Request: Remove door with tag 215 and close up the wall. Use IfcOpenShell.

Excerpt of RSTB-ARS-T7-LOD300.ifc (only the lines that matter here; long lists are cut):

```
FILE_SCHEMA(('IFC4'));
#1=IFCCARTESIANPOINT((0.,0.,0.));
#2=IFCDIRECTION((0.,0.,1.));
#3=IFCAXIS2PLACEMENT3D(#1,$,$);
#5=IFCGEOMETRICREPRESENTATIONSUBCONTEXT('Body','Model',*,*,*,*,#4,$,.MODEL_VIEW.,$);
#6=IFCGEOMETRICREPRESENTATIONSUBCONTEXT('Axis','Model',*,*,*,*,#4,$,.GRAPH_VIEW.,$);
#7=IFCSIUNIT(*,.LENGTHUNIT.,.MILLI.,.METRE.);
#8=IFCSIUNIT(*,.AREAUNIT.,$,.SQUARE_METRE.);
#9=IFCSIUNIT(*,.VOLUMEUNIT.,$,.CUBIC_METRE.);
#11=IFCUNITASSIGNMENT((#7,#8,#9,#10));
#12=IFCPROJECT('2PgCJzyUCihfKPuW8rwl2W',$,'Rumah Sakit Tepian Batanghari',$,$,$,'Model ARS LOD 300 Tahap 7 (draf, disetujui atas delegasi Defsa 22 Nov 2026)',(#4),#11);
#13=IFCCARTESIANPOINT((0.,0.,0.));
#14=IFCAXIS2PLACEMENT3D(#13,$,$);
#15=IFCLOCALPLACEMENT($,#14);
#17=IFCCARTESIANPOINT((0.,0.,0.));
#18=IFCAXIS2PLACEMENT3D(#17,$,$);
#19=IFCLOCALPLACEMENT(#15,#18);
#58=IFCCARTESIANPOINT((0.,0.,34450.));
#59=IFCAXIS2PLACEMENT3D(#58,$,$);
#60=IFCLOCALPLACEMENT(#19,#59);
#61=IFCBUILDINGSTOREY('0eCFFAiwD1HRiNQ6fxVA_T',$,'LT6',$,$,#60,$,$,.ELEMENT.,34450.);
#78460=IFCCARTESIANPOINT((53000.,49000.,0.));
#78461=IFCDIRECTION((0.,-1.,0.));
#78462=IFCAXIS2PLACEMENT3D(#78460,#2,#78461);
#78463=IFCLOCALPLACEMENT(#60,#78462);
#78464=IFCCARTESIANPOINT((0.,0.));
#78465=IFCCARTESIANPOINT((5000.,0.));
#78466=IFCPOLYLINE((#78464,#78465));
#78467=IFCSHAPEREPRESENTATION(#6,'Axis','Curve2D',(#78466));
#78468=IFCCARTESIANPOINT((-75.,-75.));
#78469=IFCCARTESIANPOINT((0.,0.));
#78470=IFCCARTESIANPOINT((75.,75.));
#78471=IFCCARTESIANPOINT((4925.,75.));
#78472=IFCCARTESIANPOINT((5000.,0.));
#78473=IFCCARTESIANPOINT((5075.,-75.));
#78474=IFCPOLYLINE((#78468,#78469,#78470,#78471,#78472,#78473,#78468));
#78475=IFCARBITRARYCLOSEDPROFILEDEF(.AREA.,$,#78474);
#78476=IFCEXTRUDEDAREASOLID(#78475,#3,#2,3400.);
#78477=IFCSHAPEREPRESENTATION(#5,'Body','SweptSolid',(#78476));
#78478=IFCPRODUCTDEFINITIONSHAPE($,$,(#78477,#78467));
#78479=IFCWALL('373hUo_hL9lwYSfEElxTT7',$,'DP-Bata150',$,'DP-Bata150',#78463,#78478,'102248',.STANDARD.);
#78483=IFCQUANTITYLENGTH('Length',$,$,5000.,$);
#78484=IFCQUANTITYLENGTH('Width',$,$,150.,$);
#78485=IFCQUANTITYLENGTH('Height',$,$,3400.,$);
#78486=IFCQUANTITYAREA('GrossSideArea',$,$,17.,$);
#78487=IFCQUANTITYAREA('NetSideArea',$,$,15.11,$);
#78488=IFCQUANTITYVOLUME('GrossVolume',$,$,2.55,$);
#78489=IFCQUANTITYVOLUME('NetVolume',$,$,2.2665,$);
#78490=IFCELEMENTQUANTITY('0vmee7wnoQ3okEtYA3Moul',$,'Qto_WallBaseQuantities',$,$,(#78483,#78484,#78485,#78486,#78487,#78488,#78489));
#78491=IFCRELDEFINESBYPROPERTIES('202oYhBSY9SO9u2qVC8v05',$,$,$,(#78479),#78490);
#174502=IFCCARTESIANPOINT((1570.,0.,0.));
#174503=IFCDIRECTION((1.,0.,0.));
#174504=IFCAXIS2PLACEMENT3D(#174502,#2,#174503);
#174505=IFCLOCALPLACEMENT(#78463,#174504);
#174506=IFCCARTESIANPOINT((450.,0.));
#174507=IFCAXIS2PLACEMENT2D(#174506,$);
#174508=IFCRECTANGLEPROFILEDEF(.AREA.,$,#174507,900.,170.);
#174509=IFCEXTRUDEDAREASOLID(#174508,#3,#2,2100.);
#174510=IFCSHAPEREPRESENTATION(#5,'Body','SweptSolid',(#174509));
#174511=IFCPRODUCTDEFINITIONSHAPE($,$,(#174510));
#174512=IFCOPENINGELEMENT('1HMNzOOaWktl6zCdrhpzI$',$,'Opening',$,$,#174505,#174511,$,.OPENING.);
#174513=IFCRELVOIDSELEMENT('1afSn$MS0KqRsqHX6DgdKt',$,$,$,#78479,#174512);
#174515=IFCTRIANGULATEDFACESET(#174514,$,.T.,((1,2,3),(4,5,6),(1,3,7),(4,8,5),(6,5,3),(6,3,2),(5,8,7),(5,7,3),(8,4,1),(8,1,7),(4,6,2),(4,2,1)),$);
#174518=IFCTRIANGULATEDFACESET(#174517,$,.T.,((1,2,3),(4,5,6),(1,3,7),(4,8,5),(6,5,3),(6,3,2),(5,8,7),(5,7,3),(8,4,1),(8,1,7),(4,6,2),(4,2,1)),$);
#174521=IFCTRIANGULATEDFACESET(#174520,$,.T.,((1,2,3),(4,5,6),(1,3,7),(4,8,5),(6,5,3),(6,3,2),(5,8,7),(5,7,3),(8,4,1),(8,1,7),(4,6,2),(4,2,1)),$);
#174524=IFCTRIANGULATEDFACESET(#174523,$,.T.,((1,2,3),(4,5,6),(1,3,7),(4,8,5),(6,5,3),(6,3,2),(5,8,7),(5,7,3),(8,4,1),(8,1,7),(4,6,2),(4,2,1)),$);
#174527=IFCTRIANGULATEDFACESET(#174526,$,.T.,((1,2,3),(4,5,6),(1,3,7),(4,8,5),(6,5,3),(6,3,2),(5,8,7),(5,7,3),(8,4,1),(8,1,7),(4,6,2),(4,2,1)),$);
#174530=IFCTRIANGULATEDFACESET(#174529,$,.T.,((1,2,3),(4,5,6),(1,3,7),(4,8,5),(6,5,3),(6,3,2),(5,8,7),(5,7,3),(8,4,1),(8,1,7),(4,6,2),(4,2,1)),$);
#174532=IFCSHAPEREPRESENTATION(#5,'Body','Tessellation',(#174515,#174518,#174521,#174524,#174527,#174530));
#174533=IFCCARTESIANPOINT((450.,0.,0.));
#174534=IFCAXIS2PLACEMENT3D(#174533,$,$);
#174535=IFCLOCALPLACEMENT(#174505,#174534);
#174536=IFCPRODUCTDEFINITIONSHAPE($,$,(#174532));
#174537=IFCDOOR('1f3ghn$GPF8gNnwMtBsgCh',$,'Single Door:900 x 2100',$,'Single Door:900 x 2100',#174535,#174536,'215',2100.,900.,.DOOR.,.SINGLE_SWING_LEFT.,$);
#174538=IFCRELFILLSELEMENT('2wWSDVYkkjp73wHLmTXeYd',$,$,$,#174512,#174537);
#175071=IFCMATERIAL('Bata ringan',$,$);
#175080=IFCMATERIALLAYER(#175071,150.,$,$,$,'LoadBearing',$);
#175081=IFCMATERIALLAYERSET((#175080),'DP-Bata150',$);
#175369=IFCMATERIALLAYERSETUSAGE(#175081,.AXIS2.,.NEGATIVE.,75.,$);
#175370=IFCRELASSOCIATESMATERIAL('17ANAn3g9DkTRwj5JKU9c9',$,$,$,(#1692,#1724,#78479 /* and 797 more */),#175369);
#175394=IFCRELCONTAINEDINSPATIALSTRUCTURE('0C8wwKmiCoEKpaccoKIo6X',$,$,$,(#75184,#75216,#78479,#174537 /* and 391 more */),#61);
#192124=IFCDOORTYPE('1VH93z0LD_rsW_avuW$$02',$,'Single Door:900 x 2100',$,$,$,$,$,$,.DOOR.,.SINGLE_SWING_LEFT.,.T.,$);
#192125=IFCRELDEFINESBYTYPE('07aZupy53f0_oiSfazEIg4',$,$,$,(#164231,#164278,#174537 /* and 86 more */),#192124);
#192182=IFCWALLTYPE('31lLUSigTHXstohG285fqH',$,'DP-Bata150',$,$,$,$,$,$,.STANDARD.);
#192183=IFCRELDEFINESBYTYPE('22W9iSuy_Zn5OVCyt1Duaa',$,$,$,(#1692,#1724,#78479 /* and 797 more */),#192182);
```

```python
import ifcopenshell
import ifcopenshell.api.feature
import ifcopenshell.api.pset
import ifcopenshell.api.root
import ifcopenshell.geom
import ifcopenshell.util.element
import ifcopenshell.util.shape
import ifcopenshell.util.unit

model = ifcopenshell.open("RSTB-ARS-T7-LOD300.ifc")
area_scale = ifcopenshell.util.unit.calculate_unit_scale(model, "AREAUNIT")
volume_scale = ifcopenshell.util.unit.calculate_unit_scale(model, "VOLUMEUNIT")
settings = ifcopenshell.geom.settings()


def volume(element):
    """Net volume in cubic metres, openings subtracted."""
    shape = ifcopenshell.geom.create_shape(settings, element)
    return ifcopenshell.util.shape.get_volume(shape.geometry)


door = model.by_id(174537)
opening = door.FillsVoids[0].RelatingOpeningElement
wall = opening.VoidsElements[0].RelatingBuildingElement
before = volume(wall)

ifcopenshell.api.root.remove_product(model, product=door)
ifcopenshell.api.feature.remove_feature(model, feature=opening)

after = volume(wall)
thickness = 0.15  # wall thickness in metres

# Update the wall's stored quantities.
qto = model.by_id(ifcopenshell.util.element.get_pset(wall, "Qto_WallBaseQuantities", should_inherit=False)["id"])
ifcopenshell.api.pset.edit_qto(model, qto=qto, properties={
    "NetSideArea": after / thickness / area_scale,
    "NetVolume": after / volume_scale,
})

print(f"wall volume {before:.3f} -> {after:.3f} m3")

model.write("RSTB-ARS-T7-LOD300_v2.ifc")
```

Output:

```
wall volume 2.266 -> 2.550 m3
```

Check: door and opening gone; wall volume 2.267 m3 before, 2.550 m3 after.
